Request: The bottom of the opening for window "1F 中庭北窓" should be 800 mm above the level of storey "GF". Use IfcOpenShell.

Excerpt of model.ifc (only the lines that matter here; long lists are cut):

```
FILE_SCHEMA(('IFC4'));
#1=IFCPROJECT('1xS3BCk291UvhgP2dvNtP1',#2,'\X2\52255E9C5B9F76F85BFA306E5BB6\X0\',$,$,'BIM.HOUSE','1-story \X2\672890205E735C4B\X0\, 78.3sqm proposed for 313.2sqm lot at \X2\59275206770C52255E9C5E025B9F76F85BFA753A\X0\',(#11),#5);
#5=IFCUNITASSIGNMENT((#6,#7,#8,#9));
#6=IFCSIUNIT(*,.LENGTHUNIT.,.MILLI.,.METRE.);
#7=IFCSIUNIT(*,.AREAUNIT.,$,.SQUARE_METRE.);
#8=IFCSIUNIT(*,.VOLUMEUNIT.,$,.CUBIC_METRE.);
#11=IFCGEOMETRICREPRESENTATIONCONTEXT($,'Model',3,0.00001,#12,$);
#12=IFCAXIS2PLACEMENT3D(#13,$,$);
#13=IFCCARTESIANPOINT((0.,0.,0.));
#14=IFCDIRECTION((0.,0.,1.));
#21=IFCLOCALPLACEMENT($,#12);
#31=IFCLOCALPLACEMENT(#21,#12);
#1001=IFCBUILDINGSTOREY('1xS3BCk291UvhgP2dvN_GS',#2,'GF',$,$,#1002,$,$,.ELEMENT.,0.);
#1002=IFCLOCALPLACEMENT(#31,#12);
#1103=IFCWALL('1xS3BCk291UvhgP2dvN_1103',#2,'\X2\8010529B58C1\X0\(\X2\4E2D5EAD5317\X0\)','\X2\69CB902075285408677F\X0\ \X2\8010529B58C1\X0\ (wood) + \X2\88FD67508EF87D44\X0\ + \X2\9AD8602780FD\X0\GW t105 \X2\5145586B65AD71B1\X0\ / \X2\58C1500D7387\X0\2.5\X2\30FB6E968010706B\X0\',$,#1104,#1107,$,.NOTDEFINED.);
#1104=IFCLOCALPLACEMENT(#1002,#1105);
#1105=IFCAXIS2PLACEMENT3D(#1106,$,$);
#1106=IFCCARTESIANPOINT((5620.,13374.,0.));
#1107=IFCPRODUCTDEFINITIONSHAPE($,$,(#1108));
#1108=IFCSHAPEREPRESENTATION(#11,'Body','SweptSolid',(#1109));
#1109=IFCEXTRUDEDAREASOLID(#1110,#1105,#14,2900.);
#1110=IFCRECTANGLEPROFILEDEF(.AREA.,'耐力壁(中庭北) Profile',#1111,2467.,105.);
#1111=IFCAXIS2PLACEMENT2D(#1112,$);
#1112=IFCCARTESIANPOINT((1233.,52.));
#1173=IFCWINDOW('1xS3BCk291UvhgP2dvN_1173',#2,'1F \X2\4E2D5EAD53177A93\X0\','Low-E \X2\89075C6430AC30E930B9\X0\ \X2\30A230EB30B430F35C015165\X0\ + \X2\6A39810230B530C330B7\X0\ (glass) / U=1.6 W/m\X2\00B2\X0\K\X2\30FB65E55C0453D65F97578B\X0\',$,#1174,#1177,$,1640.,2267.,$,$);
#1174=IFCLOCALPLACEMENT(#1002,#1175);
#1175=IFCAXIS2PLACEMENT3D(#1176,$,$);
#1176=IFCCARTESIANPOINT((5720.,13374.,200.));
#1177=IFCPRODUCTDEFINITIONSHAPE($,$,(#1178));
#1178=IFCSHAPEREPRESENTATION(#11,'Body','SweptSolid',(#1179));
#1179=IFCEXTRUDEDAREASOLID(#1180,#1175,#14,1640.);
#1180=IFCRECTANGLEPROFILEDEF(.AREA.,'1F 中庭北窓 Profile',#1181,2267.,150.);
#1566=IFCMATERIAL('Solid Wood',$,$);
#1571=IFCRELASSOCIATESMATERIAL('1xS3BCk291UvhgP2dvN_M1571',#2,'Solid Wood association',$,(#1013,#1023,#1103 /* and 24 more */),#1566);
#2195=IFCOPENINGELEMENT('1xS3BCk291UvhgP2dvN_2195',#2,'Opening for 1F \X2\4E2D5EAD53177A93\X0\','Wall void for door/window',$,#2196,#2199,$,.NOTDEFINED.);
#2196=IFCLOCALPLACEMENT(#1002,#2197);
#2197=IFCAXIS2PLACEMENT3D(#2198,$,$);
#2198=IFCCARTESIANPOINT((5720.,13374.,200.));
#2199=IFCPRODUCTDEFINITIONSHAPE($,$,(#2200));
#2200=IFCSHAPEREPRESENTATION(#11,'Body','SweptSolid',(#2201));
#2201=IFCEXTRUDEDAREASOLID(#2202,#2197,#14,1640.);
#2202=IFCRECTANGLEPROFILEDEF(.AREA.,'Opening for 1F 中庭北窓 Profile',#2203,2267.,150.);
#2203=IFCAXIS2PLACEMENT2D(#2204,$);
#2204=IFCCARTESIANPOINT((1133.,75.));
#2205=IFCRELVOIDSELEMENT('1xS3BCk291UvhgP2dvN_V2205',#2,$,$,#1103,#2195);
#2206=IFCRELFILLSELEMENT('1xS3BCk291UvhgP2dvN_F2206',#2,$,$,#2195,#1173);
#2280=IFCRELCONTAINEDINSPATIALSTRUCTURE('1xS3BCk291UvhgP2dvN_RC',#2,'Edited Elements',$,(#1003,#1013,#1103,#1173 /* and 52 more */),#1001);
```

```python
import numpy as np
import ifcopenshell
import ifcopenshell.api.geometry
import ifcopenshell.geom
import ifcopenshell.util.element
import ifcopenshell.util.placement
import ifcopenshell.util.shape
import ifcopenshell.util.unit

model = ifcopenshell.open("model.ifc")
unit_scale = ifcopenshell.util.unit.calculate_unit_scale(model)

window = model.by_guid("1xS3BCk291UvhgP2dvN_1173")
opening = window.FillsVoids[0].RelatingOpeningElement
storey = ifcopenshell.util.element.get_container(window, ifc_class="IfcBuildingStorey")
level = ifcopenshell.util.placement.get_local_placement(storey.ObjectPlacement)[2, 3]

# The opening's origin need not be at the sill, so measure its lowest point.
shape = ifcopenshell.geom.create_shape(ifcopenshell.geom.settings(), opening)
bottom = ifcopenshell.util.shape.get_shape_bottom_elevation(shape, shape.geometry) / unit_scale
dz = level + 800.0 - bottom

shift = np.array([0.0, 0.0, dz])
# The window is not placed relative to its opening, so move both.
for product in (opening, window):
    matrix = ifcopenshell.util.placement.get_local_placement(product.ObjectPlacement)
    matrix[:3, 3] += shift
    ifcopenshell.api.geometry.edit_object_placement(model, product=product, matrix=matrix, is_si=False)

print(f"moved by {dz * unit_scale:+.3f} m")

model.write("model_v2.ifc")
```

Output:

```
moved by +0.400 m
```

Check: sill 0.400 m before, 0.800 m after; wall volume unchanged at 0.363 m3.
